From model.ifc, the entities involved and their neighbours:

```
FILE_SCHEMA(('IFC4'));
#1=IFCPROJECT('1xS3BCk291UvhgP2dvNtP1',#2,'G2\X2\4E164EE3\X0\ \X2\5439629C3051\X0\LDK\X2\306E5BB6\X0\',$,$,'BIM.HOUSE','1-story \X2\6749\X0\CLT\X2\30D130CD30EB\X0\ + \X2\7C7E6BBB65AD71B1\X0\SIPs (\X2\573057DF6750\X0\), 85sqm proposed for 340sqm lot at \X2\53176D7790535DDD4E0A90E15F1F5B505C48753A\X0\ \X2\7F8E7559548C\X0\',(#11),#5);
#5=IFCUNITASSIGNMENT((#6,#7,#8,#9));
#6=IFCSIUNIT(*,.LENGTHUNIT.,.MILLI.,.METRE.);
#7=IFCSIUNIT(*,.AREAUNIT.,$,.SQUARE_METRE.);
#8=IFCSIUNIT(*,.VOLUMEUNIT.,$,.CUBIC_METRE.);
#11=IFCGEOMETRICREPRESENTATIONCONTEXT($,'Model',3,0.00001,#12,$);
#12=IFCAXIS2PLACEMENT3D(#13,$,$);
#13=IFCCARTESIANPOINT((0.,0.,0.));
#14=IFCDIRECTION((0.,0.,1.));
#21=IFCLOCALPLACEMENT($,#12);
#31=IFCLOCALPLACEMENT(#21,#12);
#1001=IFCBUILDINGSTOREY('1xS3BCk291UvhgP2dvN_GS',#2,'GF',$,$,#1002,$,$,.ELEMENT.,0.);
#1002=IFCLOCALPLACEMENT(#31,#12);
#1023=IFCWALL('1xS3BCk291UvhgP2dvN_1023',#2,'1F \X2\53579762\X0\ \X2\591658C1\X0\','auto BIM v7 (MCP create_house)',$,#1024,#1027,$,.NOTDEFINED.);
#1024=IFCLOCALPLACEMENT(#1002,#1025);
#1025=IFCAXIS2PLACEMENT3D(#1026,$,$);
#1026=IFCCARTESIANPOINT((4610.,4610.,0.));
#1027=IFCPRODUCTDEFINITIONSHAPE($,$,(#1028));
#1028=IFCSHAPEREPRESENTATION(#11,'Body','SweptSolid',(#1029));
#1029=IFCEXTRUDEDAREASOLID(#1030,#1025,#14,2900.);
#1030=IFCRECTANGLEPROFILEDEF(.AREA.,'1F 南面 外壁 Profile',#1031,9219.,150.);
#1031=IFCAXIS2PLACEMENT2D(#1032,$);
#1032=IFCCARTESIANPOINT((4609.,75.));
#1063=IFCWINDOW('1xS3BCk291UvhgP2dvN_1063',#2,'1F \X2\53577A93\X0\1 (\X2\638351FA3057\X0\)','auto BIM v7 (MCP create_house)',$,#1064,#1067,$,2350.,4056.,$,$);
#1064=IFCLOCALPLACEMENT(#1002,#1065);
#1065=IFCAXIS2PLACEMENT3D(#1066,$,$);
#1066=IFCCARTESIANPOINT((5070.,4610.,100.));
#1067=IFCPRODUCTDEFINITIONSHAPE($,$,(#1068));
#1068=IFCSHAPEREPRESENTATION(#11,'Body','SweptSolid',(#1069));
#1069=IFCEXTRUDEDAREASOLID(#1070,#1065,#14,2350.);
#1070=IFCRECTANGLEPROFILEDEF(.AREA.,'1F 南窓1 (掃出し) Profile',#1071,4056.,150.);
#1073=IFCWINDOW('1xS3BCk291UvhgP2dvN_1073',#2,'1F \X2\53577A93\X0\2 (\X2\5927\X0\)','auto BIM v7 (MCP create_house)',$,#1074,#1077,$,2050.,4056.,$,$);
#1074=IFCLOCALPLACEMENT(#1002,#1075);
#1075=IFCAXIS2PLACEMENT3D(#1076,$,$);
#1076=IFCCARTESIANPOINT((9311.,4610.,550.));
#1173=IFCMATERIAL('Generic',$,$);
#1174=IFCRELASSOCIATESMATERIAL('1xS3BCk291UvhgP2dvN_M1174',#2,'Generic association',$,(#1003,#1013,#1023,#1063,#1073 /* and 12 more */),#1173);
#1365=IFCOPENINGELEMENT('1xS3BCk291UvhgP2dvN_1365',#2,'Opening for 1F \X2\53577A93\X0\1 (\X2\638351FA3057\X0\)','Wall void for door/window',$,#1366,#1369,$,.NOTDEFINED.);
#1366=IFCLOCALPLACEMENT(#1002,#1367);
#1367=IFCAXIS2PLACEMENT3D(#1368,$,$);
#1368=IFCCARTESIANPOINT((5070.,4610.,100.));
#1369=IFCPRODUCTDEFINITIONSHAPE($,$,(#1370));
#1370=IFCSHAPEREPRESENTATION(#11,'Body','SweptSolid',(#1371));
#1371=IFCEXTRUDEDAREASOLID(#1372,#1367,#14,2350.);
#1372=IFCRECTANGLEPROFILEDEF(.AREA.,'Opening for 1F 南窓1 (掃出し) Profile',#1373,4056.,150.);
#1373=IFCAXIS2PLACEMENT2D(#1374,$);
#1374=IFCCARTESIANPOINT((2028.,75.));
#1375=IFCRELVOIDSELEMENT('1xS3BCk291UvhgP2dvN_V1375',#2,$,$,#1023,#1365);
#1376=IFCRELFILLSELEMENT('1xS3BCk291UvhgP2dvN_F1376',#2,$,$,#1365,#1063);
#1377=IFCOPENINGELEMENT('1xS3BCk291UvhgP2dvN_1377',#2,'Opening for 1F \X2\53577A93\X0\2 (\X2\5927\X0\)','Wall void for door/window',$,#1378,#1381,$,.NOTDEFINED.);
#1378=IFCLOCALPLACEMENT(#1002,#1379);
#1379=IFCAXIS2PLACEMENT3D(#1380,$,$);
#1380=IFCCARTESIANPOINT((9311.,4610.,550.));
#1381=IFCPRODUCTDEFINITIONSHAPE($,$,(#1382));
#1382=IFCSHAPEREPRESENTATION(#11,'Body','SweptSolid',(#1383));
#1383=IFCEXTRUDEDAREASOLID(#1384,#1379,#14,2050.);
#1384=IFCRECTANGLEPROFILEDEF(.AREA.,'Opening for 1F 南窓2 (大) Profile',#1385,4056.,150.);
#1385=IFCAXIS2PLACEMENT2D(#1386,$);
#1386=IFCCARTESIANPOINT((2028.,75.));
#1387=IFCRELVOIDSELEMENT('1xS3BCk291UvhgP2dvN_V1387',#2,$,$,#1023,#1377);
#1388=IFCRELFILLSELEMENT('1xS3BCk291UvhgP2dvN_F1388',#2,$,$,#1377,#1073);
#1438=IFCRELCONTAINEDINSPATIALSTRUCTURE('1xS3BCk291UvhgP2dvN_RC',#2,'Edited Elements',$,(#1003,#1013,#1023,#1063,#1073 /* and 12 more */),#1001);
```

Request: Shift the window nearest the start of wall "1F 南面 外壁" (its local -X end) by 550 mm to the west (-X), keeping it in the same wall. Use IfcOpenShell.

```python
import ifcopenshell
import ifcopenshell.api.geometry
import ifcopenshell.util.placement
import ifcopenshell.util.unit

model = ifcopenshell.open("model.ifc")
unit_scale = ifcopenshell.util.unit.calculate_unit_scale(model)

window = model.by_guid("1xS3BCk291UvhgP2dvN_1063")
opening = window.FillsVoids[0].RelatingOpeningElement
wall = opening.VoidsElements[0].RelatingBuildingElement

wall_matrix = ifcopenshell.util.placement.get_local_placement(wall.ObjectPlacement)
shift = wall_matrix[:3, 0] * -0.55 / unit_scale
before = ifcopenshell.util.placement.get_local_placement(window.ObjectPlacement)[:3, 3].copy()

# The window is not placed relative to its opening, so move both.
for product in (opening, window):
    matrix = ifcopenshell.util.placement.get_local_placement(product.ObjectPlacement)
    matrix[:3, 3] += shift
    ifcopenshell.api.geometry.edit_object_placement(model, product=product, matrix=matrix, is_si=False)

after = ifcopenshell.util.placement.get_local_placement(window.ObjectPlacement)[:3, 3]
print("window moved by", (after - before).round(3) + 0.0)

model.write("model_edited.ifc")
```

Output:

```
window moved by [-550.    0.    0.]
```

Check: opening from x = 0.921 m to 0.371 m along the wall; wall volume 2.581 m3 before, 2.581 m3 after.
